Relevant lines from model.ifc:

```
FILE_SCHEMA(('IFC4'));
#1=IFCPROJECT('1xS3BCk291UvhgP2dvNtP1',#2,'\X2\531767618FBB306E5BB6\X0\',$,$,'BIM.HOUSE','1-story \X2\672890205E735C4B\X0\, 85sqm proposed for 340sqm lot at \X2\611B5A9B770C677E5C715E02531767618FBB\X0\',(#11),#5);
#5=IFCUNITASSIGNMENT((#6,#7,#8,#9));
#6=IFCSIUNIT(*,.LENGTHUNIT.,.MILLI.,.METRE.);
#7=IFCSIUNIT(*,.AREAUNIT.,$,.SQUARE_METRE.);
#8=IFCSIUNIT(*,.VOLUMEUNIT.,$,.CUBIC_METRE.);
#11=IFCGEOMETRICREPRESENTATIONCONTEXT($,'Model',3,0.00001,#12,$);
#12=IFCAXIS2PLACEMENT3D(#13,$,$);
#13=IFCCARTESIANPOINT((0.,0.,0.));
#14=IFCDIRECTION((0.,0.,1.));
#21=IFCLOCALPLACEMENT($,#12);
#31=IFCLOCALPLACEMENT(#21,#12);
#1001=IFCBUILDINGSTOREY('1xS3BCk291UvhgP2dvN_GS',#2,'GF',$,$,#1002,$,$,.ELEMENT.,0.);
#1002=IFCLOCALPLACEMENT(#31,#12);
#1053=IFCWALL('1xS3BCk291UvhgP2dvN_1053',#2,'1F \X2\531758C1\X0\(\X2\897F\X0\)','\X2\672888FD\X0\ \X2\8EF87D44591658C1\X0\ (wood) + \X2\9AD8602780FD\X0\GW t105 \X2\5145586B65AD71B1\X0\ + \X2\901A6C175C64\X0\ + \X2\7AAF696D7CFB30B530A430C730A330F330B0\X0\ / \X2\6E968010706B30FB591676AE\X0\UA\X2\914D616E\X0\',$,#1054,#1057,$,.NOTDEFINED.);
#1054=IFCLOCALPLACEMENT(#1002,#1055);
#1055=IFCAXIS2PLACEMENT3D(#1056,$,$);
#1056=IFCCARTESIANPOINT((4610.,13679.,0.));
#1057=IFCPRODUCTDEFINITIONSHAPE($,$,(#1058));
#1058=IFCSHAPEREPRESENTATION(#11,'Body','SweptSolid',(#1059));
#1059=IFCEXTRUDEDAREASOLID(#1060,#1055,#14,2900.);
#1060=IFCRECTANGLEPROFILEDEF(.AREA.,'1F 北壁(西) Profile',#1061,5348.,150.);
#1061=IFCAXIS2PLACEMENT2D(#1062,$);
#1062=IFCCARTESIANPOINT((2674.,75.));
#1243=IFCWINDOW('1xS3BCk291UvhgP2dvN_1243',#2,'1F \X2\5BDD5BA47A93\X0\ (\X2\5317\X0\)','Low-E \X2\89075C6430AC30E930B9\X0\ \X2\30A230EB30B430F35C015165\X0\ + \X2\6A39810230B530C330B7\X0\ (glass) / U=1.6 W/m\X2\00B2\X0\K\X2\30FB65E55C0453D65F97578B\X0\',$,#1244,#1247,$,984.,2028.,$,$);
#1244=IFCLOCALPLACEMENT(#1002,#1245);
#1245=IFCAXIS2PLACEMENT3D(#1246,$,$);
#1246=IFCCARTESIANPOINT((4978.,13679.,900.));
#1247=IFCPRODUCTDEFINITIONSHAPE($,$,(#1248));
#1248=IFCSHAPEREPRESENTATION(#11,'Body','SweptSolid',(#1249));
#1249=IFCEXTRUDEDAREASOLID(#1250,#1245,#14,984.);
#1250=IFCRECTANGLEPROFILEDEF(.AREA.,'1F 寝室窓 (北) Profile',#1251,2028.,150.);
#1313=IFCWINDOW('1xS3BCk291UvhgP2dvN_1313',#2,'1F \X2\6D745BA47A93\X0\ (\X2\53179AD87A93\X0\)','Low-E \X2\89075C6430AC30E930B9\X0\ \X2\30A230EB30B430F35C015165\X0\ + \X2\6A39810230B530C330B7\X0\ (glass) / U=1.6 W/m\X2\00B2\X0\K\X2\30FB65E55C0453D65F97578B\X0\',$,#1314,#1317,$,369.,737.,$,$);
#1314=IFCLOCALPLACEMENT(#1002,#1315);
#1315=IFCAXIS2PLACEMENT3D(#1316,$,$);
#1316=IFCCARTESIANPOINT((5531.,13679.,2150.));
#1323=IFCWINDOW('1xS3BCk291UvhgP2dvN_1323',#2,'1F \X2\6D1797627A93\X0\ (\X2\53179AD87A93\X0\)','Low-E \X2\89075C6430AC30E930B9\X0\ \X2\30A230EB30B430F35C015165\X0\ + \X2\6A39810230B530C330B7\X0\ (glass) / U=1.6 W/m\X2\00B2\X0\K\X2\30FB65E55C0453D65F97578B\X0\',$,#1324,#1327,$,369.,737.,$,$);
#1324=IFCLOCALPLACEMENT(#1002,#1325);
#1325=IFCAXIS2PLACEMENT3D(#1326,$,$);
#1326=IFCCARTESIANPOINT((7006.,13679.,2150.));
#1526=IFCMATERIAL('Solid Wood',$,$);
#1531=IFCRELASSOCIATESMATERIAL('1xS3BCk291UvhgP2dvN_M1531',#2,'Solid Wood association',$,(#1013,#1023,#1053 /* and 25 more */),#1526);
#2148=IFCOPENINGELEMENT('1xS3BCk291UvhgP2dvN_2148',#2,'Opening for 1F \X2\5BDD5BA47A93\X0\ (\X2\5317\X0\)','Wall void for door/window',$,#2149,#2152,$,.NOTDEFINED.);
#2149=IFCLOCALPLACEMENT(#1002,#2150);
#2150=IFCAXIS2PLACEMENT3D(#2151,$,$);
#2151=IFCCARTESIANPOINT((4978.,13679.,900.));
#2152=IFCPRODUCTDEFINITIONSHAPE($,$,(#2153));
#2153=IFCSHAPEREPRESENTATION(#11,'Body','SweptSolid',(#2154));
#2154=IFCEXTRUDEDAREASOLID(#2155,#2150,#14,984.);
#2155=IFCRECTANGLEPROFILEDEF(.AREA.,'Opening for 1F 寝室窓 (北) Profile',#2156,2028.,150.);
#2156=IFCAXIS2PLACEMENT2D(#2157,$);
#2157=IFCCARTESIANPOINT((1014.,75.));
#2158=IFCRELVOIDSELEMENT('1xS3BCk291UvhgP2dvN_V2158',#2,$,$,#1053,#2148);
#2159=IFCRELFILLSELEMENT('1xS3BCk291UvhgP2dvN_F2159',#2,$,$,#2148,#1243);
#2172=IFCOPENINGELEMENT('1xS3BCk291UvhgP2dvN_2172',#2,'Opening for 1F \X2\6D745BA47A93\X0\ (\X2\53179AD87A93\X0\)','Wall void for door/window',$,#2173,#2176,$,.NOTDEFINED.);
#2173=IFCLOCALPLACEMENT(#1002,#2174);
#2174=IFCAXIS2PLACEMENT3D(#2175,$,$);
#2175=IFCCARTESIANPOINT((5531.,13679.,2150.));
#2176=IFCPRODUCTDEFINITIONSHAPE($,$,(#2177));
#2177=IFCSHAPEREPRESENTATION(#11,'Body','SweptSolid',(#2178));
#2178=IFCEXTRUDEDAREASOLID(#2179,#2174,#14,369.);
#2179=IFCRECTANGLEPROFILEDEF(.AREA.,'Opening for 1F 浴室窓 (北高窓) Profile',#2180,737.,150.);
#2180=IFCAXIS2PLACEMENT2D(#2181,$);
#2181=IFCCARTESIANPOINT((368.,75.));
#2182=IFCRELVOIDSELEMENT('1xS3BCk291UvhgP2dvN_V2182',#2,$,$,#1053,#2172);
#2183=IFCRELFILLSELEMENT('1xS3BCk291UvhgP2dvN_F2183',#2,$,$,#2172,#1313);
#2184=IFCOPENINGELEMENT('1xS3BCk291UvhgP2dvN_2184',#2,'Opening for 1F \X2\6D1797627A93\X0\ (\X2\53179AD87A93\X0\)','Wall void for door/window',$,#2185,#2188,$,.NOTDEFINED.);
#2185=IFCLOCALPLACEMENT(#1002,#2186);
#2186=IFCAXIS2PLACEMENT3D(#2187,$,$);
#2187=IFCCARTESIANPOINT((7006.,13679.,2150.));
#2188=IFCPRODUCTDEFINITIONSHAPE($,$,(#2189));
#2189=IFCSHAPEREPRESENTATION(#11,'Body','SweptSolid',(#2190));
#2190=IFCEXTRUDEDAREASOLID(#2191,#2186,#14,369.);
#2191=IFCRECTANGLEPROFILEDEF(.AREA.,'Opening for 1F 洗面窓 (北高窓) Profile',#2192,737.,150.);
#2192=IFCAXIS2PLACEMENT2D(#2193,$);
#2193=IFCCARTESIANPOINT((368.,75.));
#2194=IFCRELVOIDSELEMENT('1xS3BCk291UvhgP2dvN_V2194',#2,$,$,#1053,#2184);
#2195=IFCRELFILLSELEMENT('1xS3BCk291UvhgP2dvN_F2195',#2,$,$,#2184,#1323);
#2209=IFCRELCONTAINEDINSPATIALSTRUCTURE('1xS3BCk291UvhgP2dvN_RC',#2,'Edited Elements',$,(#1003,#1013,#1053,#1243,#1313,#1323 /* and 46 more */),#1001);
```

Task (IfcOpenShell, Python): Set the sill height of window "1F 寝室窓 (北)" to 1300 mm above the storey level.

```python
import numpy as np
import ifcopenshell
import ifcopenshell.api.geometry
import ifcopenshell.geom
import ifcopenshell.util.element
import ifcopenshell.util.placement
import ifcopenshell.util.shape
import ifcopenshell.util.unit

model = ifcopenshell.open("model.ifc")
unit_scale = ifcopenshell.util.unit.calculate_unit_scale(model)

window = model.by_id(1243)
opening = window.FillsVoids[0].RelatingOpeningElement
storey = ifcopenshell.util.element.get_container(window, ifc_class="IfcBuildingStorey")
level = ifcopenshell.util.placement.get_local_placement(storey.ObjectPlacement)[2, 3]

# The opening's origin need not be at the sill, so measure its lowest point.
shape = ifcopenshell.geom.create_shape(ifcopenshell.geom.settings(), opening)
bottom = ifcopenshell.util.shape.get_shape_bottom_elevation(shape, shape.geometry) / unit_scale
dz = level + 1300.0 - bottom

shift = np.array([0.0, 0.0, dz])
# The window is not placed relative to its opening, so move both.
for product in (opening, window):
    matrix = ifcopenshell.util.placement.get_local_placement(product.ObjectPlacement)
    matrix[:3, 3] += shift
    ifcopenshell.api.geometry.edit_object_placement(model, product=product, matrix=matrix, is_si=False)

print(f"moved by {dz * unit_scale:+.3f} m")

model.write("model_v2.ifc")
```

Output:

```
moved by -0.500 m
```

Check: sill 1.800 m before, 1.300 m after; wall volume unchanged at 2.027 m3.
